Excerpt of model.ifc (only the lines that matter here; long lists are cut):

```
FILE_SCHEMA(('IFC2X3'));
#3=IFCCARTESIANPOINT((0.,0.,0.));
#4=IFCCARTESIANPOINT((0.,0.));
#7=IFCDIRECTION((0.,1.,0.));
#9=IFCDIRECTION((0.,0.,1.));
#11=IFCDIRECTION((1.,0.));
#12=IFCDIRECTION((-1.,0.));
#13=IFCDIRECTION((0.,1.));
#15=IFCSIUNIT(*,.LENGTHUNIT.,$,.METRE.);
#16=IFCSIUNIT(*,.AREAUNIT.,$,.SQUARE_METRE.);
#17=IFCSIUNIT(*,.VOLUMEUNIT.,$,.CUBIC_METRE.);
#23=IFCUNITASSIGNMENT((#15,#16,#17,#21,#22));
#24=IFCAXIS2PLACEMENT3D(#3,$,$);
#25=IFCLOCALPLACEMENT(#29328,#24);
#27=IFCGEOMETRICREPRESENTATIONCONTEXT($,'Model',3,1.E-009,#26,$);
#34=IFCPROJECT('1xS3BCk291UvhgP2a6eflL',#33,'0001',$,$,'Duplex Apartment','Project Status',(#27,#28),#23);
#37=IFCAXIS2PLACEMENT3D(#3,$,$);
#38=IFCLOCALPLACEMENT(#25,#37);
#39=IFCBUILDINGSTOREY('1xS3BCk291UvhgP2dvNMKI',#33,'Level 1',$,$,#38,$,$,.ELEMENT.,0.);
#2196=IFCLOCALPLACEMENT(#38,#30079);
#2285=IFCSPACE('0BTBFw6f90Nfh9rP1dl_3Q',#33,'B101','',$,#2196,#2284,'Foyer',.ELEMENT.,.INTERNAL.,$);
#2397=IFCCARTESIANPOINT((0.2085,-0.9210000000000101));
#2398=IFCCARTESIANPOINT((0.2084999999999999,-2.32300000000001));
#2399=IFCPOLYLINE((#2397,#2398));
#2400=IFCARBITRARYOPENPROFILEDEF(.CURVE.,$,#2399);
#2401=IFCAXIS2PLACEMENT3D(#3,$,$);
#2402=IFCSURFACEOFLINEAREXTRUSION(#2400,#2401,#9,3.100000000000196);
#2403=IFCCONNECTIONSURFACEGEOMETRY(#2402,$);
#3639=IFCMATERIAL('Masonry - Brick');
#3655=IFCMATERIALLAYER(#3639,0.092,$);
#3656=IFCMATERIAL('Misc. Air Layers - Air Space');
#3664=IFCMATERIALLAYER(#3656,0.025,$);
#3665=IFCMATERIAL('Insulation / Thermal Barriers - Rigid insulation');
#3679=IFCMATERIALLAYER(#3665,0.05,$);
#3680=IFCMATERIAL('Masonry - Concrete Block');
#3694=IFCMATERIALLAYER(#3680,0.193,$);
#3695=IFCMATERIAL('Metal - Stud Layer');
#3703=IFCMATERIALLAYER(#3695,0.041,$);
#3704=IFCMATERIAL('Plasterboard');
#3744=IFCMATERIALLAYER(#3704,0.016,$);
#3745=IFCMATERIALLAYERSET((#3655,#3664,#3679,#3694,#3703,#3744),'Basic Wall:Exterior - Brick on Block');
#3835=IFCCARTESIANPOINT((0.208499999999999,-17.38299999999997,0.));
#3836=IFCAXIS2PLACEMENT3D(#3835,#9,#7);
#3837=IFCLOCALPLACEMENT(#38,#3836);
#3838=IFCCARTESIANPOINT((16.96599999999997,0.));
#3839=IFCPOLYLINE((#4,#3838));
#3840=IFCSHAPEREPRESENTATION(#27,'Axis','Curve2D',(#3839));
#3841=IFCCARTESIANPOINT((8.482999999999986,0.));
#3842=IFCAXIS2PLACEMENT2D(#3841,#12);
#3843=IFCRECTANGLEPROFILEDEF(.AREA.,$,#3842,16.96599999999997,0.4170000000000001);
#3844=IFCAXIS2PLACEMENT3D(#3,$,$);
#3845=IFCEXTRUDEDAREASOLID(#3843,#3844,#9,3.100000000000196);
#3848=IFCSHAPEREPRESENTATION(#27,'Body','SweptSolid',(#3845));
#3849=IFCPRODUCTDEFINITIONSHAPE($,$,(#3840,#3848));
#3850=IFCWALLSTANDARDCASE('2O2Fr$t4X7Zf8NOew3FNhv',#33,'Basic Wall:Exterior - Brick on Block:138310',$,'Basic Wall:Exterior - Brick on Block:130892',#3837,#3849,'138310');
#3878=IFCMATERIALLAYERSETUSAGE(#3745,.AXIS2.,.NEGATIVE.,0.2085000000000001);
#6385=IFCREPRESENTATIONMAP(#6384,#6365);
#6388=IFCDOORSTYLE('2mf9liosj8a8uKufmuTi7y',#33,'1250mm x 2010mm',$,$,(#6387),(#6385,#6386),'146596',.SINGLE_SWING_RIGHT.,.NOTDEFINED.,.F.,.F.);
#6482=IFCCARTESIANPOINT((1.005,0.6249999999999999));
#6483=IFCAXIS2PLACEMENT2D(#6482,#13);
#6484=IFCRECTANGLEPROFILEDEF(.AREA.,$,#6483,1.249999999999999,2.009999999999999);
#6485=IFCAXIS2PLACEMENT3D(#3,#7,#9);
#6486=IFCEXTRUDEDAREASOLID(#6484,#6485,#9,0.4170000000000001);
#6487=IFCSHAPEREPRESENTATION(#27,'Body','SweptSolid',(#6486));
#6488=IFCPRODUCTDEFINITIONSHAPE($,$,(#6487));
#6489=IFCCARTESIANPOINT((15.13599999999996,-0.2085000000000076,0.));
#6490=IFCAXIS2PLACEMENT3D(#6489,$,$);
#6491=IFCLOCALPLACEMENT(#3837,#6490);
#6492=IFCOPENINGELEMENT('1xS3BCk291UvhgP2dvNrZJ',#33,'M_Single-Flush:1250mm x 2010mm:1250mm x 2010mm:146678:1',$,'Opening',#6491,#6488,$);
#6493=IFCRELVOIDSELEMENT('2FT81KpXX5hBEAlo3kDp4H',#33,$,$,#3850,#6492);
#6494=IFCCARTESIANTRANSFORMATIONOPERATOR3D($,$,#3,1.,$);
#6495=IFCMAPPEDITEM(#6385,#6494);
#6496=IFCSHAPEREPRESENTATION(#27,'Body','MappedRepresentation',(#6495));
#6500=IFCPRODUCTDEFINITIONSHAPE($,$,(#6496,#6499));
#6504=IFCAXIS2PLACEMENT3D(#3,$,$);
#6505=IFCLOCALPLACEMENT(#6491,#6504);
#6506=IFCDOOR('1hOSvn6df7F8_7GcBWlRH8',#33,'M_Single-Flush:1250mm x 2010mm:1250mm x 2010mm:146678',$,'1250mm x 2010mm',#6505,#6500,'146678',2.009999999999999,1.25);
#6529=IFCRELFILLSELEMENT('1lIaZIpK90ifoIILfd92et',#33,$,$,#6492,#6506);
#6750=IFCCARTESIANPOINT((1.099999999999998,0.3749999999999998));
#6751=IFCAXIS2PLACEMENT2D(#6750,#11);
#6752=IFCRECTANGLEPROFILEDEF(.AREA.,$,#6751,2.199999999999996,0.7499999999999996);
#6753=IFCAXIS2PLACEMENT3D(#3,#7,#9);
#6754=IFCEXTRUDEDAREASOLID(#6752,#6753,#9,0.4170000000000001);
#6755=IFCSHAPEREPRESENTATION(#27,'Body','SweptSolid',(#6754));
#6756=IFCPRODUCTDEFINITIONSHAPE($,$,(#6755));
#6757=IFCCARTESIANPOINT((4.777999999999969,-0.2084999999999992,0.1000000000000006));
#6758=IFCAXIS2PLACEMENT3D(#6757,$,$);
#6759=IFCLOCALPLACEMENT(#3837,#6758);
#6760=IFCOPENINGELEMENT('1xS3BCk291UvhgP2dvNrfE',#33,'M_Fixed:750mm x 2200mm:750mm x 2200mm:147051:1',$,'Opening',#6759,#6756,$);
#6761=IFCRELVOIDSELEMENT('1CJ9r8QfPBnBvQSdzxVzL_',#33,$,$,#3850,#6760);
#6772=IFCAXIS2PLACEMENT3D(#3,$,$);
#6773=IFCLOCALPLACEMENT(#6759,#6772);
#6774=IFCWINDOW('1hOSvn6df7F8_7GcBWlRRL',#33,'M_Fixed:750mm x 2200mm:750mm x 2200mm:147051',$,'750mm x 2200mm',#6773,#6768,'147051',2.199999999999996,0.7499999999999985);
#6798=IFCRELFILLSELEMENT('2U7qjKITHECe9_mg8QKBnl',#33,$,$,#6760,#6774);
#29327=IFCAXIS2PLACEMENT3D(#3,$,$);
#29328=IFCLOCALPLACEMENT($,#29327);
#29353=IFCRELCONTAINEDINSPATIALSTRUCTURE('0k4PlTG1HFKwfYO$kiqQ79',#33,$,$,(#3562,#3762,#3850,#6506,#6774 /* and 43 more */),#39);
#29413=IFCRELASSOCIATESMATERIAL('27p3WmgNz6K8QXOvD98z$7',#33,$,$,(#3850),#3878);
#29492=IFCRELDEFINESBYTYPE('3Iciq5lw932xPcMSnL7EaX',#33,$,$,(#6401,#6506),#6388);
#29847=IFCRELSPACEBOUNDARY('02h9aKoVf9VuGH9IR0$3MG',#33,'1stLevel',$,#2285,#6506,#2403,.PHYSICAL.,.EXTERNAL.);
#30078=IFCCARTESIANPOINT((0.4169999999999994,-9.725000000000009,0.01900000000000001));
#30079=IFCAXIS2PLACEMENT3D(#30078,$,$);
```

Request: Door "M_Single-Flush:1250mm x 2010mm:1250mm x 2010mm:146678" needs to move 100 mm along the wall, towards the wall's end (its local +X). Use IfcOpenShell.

```python
import numpy as np
import ifcopenshell
import ifcopenshell.api.geometry
import ifcopenshell.util.placement
import ifcopenshell.util.unit

model = ifcopenshell.open("model.ifc")
unit_scale = ifcopenshell.util.unit.calculate_unit_scale(model)

door = model.by_guid("1hOSvn6df7F8_7GcBWlRH8")
opening = door.FillsVoids[0].RelatingOpeningElement
wall = opening.VoidsElements[0].RelatingBuildingElement

wall_matrix = ifcopenshell.util.placement.get_local_placement(wall.ObjectPlacement)
shift = wall_matrix[:3, 0] * 0.1 / unit_scale
before = ifcopenshell.util.placement.get_local_placement(door.ObjectPlacement)[:3, 3].copy()

# The door is placed relative to its opening, so it follows when the opening moves.
matrix = ifcopenshell.util.placement.get_local_placement(opening.ObjectPlacement)
matrix[:3, 3] += shift
ifcopenshell.api.geometry.edit_object_placement(
    model, product=opening, matrix=matrix, is_si=False, should_transform_children=True
)

# Space boundary surfaces are stored in each space's coordinates; move them too.
for rel in door.ProvidesBoundaries:
    if not rel.ConnectionGeometry:
        continue
    surface = rel.ConnectionGeometry.SurfaceOnRelatingElement
    space_matrix = ifcopenshell.util.placement.get_local_placement(rel.RelatingSpace.ObjectPlacement)
    point = np.array(surface.Position.Location.Coordinates) + space_matrix[:3, :3].T @ shift
    surface.Position = model.createIfcAxis2Placement3D(
        model.createIfcCartesianPoint(point.tolist()), surface.Position.Axis, surface.Position.RefDirection
    )

after = ifcopenshell.util.placement.get_local_placement(door.ObjectPlacement)[:3, 3]
print("door moved by", (after - before).round(3) + 0.0)

model.write("model_edited.ifc")
```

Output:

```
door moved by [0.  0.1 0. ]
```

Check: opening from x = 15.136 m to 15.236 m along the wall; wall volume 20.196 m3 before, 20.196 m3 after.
